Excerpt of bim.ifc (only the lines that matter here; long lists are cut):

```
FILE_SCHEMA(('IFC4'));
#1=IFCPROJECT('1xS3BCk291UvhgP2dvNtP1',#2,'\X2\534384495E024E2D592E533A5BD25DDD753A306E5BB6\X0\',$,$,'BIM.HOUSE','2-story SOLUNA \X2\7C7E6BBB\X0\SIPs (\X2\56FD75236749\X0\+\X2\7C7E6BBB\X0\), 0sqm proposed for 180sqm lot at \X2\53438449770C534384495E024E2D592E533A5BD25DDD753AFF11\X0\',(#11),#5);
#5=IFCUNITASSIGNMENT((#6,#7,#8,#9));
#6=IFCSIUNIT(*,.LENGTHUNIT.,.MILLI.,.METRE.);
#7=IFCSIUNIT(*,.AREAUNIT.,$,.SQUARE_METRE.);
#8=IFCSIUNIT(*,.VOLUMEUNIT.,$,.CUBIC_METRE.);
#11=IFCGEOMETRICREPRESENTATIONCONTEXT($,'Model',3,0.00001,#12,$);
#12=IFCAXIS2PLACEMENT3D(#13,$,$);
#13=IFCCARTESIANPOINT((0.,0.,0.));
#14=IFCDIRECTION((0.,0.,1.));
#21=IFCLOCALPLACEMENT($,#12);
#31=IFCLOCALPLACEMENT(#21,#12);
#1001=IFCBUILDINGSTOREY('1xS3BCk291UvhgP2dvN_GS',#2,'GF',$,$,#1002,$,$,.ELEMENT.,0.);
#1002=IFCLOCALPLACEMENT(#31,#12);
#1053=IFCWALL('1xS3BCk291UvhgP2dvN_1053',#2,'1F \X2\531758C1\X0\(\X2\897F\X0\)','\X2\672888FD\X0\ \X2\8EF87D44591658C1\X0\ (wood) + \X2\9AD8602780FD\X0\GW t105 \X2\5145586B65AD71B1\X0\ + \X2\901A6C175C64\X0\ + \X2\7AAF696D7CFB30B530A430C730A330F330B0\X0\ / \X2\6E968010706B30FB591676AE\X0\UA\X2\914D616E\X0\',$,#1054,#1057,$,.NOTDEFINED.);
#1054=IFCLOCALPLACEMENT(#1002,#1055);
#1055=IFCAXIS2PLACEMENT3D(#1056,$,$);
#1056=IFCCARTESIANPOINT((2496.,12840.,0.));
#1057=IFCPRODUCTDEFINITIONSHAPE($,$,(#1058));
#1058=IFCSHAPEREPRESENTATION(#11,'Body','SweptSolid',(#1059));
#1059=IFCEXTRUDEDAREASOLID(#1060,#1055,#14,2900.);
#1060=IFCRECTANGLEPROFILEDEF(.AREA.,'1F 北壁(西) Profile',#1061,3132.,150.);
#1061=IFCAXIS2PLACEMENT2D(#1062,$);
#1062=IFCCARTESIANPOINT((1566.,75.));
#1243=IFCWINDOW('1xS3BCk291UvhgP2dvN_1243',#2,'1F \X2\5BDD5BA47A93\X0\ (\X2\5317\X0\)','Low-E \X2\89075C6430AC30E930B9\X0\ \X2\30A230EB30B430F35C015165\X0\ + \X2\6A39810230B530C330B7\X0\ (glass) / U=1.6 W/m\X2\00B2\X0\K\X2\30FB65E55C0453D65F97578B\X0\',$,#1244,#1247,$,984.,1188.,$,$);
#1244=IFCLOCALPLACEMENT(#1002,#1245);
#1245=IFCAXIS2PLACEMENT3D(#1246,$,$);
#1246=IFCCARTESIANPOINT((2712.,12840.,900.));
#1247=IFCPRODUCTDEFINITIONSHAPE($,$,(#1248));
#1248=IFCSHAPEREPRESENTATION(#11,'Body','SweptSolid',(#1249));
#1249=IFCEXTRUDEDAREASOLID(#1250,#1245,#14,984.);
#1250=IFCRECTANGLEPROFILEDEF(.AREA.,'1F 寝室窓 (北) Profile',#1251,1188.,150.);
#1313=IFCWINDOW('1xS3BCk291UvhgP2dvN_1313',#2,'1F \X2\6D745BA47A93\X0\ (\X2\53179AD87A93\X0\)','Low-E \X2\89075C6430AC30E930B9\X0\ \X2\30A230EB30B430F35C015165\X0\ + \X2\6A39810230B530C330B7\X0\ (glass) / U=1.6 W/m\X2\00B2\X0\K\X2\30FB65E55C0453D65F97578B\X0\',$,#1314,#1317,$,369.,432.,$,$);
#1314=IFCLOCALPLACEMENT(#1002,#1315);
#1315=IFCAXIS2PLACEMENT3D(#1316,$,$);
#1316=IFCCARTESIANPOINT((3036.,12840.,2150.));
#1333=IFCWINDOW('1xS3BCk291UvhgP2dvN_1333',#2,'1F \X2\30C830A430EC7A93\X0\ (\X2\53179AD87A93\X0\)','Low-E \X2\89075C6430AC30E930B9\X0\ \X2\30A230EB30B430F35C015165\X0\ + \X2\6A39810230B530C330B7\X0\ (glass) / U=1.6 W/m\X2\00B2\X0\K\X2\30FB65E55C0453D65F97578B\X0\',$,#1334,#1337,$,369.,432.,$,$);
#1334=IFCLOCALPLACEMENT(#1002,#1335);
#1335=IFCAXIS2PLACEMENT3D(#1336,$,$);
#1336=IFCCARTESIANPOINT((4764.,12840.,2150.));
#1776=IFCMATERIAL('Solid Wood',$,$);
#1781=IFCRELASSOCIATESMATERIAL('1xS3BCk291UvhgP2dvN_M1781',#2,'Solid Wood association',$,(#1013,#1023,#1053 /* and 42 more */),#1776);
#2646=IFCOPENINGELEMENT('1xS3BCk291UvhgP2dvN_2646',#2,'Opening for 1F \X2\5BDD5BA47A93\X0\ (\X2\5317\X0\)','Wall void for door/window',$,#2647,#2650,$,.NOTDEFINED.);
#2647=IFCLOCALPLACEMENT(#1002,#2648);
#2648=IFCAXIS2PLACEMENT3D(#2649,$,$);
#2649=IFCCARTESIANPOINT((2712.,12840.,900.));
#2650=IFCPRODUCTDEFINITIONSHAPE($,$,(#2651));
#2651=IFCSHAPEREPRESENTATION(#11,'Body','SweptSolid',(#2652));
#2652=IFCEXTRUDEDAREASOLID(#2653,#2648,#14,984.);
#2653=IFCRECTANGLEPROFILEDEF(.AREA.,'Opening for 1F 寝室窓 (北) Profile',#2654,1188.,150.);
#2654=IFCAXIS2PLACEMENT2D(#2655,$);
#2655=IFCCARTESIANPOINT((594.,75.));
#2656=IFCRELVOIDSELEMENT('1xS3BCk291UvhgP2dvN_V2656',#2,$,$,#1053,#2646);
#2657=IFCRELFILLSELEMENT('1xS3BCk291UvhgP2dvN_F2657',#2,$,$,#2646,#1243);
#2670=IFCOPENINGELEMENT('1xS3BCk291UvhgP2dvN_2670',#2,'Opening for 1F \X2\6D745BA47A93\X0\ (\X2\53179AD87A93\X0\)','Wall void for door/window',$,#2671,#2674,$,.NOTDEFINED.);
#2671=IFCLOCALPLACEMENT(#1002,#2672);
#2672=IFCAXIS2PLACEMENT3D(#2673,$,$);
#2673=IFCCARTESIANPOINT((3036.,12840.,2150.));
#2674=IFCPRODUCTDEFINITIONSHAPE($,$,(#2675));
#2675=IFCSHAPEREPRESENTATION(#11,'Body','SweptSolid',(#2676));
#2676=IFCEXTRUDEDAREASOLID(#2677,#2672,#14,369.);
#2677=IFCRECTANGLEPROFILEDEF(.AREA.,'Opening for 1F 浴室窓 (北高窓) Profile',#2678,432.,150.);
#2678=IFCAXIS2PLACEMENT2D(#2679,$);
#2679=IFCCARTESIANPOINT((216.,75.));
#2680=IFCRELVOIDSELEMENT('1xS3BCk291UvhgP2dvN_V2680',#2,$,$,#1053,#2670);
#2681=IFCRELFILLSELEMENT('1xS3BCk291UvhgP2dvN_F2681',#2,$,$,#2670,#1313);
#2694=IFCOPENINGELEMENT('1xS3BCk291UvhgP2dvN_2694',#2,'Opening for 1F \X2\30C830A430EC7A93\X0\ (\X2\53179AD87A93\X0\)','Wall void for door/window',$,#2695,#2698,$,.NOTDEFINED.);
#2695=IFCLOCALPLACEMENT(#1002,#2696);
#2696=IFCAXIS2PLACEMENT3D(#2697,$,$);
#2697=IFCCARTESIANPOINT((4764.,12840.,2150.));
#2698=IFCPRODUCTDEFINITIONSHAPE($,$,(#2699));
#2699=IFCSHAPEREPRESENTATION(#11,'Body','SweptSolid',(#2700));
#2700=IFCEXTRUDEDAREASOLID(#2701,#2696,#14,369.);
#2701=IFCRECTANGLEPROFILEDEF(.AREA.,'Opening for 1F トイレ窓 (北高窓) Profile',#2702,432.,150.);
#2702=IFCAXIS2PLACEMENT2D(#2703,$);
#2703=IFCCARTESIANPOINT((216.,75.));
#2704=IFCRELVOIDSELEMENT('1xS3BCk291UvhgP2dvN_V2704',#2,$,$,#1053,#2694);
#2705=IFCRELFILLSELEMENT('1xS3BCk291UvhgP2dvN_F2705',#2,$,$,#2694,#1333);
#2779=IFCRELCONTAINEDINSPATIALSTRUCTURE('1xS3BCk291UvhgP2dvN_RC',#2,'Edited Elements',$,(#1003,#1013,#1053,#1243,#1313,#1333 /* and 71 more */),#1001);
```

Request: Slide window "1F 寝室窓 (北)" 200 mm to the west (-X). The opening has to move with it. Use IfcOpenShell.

```python
import ifcopenshell
import ifcopenshell.api.geometry
import ifcopenshell.util.placement
import ifcopenshell.util.unit

model = ifcopenshell.open("bim.ifc")
unit_scale = ifcopenshell.util.unit.calculate_unit_scale(model)

window = model.by_guid("1xS3BCk291UvhgP2dvN_1243")
opening = window.FillsVoids[0].RelatingOpeningElement
wall = opening.VoidsElements[0].RelatingBuildingElement

wall_matrix = ifcopenshell.util.placement.get_local_placement(wall.ObjectPlacement)
shift = wall_matrix[:3, 0] * -0.2 / unit_scale
before = ifcopenshell.util.placement.get_local_placement(window.ObjectPlacement)[:3, 3].copy()

# The window is not placed relative to its opening, so move both.
for product in (opening, window):
    matrix = ifcopenshell.util.placement.get_local_placement(product.ObjectPlacement)
    matrix[:3, 3] += shift
    ifcopenshell.api.geometry.edit_object_placement(model, product=product, matrix=matrix, is_si=False)

after = ifcopenshell.util.placement.get_local_placement(window.ObjectPlacement)[:3, 3]
print("window moved by", (after - before).round(3) + 0.0)

model.write("bim-out.ifc")
```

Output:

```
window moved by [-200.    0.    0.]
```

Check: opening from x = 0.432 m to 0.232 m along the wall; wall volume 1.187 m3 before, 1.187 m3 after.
